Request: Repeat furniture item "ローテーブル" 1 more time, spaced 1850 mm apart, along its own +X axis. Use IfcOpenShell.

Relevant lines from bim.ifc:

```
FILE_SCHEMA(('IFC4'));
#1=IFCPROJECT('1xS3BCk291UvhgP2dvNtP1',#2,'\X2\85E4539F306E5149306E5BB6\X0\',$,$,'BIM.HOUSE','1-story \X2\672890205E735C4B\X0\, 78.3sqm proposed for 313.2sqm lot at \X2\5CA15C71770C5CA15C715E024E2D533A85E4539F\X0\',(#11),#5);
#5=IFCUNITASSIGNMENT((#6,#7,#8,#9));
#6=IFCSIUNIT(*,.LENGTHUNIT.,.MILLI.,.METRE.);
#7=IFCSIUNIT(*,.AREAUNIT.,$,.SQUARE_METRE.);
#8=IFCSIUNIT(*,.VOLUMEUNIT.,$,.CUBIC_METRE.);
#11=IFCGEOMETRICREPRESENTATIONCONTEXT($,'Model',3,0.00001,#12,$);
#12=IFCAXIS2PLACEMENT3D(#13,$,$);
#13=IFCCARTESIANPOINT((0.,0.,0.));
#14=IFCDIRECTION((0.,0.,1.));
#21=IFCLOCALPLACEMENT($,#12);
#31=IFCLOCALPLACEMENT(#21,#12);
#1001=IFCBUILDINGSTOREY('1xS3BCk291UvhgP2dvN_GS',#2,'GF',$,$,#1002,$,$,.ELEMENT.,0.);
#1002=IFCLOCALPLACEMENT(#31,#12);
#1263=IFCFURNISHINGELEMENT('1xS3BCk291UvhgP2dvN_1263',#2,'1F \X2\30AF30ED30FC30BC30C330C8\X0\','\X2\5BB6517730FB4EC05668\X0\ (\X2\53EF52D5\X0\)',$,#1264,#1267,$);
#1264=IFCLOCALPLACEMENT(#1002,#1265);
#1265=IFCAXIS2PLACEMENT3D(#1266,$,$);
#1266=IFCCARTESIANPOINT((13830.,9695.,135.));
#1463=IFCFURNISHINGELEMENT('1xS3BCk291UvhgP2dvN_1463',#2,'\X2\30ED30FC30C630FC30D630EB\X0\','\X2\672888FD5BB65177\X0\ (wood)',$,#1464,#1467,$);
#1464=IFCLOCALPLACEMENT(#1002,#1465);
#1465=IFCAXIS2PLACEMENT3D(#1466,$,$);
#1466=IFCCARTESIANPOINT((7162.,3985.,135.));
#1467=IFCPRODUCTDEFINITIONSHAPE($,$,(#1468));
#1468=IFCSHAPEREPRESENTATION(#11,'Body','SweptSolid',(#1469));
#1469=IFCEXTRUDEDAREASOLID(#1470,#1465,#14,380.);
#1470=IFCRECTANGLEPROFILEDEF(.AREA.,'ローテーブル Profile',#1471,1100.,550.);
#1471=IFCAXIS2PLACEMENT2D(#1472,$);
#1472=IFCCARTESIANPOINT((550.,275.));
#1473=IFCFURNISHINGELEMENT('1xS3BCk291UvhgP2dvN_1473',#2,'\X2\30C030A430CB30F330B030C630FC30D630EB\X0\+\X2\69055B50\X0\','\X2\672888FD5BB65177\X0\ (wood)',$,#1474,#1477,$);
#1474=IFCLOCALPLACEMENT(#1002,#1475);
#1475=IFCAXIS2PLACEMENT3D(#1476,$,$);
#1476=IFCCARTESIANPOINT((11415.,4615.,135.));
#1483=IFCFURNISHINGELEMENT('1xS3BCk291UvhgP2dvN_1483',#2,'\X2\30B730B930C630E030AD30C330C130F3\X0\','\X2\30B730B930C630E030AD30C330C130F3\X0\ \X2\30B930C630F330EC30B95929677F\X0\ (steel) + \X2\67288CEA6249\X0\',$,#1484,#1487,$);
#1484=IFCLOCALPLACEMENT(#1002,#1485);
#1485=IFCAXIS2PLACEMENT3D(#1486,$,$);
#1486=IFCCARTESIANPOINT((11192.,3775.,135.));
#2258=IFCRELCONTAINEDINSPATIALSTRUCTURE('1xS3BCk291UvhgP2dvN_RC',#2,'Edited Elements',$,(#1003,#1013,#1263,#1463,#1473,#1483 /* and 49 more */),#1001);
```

```python
import ifcopenshell
import ifcopenshell.api.geometry
import ifcopenshell.api.root
import ifcopenshell.util.element
import ifcopenshell.util.placement
import ifcopenshell.util.unit

model = ifcopenshell.open("bim.ifc")
unit_scale = ifcopenshell.util.unit.calculate_unit_scale(model)


def reuse_history(source, copy):
    """copy_class also copies each property set's owner history, people and application; keep the originals."""
    for rel in copy.IsDefinedBy:
        if rel.is_a("IfcRelDefinesByProperties") and (history := rel.RelatingPropertyDefinition.OwnerHistory):
            rel.RelatingPropertyDefinition.OwnerHistory = source.OwnerHistory
            ifcopenshell.util.element.remove_deep2(model, history)


source = model.by_guid("1xS3BCk291UvhgP2dvN_1463")
base = ifcopenshell.util.placement.get_local_placement(source.ObjectPlacement)
step = base[:3, 0] * 1.85 / unit_scale

for i in range(1, 2):
    copy = ifcopenshell.api.root.copy_class(model, product=source)
    copy.Representation = ifcopenshell.util.element.copy_deep(
        model, source.Representation, exclude=["IfcGeometricRepresentationContext", "IfcRepresentationMap"]
    )
    reuse_history(source, copy)
    matrix = base.copy()
    matrix[:3, 3] += i * step
    print("added at", matrix[:3, 3].round(3) + 0.0)
    ifcopenshell.api.geometry.edit_object_placement(model, product=copy, matrix=matrix, is_si=False)

model.write("bim_updated.ifc")
```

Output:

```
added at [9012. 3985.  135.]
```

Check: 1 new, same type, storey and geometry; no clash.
